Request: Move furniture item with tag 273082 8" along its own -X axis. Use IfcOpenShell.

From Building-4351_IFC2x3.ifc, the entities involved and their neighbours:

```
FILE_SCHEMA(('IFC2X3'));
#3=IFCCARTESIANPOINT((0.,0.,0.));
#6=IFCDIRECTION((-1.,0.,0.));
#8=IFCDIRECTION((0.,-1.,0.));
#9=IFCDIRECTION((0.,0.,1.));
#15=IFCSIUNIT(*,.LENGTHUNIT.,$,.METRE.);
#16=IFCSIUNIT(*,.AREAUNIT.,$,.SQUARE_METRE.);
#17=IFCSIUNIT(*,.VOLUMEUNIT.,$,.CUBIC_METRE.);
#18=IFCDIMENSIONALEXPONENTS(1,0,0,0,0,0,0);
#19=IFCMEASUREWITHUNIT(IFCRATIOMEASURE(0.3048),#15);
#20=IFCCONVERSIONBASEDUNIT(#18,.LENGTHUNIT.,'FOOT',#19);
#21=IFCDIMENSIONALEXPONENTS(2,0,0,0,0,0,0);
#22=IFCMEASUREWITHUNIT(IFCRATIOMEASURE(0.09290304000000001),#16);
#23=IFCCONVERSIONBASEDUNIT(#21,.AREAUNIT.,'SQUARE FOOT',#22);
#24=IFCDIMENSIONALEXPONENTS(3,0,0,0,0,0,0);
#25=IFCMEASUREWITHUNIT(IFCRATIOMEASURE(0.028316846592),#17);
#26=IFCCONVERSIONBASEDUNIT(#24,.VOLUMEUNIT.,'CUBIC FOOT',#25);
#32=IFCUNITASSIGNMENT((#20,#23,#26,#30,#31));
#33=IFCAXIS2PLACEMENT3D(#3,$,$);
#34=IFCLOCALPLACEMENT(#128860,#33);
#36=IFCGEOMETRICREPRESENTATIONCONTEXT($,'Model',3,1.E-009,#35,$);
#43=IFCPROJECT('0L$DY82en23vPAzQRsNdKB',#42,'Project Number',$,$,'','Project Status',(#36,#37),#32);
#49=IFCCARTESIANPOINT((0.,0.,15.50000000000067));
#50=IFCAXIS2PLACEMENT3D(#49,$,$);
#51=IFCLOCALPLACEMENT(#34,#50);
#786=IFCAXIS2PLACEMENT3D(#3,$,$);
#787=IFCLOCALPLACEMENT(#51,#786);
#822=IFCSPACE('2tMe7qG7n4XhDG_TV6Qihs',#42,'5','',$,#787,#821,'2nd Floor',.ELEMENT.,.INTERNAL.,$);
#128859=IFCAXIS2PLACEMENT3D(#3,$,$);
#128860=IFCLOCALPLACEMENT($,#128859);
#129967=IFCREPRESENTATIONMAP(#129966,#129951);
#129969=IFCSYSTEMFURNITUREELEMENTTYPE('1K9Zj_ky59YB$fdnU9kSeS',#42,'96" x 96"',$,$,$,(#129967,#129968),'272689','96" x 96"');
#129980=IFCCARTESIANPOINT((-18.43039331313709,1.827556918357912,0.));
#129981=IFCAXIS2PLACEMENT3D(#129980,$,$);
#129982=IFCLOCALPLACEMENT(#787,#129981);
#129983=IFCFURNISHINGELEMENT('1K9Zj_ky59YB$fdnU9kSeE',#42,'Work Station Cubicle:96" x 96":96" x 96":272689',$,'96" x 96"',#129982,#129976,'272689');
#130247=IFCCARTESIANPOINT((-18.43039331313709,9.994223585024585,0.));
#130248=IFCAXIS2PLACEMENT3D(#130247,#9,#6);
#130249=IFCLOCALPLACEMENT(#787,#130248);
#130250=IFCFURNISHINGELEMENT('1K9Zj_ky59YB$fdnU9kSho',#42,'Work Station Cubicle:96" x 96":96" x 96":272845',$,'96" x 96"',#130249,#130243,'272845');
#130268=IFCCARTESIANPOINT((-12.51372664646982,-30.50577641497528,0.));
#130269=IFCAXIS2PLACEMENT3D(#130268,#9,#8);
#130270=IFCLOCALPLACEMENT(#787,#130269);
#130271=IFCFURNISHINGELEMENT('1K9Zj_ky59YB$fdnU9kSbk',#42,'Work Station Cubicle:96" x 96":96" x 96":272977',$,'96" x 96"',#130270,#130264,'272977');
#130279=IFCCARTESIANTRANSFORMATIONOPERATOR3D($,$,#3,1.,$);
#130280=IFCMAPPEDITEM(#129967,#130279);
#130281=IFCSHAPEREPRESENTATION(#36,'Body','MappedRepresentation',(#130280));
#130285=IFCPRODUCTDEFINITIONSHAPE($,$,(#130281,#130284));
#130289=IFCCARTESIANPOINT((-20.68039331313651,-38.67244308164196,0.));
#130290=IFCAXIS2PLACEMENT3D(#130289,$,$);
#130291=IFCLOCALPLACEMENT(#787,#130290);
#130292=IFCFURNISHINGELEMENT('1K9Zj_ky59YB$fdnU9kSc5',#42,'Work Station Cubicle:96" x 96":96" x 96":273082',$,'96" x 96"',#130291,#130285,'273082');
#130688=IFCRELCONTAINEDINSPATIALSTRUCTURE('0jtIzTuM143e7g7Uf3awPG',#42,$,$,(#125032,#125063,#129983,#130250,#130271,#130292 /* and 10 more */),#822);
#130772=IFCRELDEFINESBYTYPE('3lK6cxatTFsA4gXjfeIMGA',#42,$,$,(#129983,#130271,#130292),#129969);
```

```python
import ifcopenshell
import ifcopenshell.api.geometry
import ifcopenshell.util.placement
import ifcopenshell.util.unit

model = ifcopenshell.open("Building-4351_IFC2x3.ifc")
unit_scale = ifcopenshell.util.unit.calculate_unit_scale(model)

item = model.by_id(130292)
matrix = ifcopenshell.util.placement.get_local_placement(item.ObjectPlacement)
matrix[:3, 3] -= matrix[:3, 0] * 8 * 0.0254 / unit_scale
ifcopenshell.api.geometry.edit_object_placement(model, product=item, matrix=matrix, is_si=False)

print(ifcopenshell.util.placement.get_local_placement(item.ObjectPlacement).round(3) + 0.0)

model.write("Building-4351_IFC2x3_edited.ifc")
```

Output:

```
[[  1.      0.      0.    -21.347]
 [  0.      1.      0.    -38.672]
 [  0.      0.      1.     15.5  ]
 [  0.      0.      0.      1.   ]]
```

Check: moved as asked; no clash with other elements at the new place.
